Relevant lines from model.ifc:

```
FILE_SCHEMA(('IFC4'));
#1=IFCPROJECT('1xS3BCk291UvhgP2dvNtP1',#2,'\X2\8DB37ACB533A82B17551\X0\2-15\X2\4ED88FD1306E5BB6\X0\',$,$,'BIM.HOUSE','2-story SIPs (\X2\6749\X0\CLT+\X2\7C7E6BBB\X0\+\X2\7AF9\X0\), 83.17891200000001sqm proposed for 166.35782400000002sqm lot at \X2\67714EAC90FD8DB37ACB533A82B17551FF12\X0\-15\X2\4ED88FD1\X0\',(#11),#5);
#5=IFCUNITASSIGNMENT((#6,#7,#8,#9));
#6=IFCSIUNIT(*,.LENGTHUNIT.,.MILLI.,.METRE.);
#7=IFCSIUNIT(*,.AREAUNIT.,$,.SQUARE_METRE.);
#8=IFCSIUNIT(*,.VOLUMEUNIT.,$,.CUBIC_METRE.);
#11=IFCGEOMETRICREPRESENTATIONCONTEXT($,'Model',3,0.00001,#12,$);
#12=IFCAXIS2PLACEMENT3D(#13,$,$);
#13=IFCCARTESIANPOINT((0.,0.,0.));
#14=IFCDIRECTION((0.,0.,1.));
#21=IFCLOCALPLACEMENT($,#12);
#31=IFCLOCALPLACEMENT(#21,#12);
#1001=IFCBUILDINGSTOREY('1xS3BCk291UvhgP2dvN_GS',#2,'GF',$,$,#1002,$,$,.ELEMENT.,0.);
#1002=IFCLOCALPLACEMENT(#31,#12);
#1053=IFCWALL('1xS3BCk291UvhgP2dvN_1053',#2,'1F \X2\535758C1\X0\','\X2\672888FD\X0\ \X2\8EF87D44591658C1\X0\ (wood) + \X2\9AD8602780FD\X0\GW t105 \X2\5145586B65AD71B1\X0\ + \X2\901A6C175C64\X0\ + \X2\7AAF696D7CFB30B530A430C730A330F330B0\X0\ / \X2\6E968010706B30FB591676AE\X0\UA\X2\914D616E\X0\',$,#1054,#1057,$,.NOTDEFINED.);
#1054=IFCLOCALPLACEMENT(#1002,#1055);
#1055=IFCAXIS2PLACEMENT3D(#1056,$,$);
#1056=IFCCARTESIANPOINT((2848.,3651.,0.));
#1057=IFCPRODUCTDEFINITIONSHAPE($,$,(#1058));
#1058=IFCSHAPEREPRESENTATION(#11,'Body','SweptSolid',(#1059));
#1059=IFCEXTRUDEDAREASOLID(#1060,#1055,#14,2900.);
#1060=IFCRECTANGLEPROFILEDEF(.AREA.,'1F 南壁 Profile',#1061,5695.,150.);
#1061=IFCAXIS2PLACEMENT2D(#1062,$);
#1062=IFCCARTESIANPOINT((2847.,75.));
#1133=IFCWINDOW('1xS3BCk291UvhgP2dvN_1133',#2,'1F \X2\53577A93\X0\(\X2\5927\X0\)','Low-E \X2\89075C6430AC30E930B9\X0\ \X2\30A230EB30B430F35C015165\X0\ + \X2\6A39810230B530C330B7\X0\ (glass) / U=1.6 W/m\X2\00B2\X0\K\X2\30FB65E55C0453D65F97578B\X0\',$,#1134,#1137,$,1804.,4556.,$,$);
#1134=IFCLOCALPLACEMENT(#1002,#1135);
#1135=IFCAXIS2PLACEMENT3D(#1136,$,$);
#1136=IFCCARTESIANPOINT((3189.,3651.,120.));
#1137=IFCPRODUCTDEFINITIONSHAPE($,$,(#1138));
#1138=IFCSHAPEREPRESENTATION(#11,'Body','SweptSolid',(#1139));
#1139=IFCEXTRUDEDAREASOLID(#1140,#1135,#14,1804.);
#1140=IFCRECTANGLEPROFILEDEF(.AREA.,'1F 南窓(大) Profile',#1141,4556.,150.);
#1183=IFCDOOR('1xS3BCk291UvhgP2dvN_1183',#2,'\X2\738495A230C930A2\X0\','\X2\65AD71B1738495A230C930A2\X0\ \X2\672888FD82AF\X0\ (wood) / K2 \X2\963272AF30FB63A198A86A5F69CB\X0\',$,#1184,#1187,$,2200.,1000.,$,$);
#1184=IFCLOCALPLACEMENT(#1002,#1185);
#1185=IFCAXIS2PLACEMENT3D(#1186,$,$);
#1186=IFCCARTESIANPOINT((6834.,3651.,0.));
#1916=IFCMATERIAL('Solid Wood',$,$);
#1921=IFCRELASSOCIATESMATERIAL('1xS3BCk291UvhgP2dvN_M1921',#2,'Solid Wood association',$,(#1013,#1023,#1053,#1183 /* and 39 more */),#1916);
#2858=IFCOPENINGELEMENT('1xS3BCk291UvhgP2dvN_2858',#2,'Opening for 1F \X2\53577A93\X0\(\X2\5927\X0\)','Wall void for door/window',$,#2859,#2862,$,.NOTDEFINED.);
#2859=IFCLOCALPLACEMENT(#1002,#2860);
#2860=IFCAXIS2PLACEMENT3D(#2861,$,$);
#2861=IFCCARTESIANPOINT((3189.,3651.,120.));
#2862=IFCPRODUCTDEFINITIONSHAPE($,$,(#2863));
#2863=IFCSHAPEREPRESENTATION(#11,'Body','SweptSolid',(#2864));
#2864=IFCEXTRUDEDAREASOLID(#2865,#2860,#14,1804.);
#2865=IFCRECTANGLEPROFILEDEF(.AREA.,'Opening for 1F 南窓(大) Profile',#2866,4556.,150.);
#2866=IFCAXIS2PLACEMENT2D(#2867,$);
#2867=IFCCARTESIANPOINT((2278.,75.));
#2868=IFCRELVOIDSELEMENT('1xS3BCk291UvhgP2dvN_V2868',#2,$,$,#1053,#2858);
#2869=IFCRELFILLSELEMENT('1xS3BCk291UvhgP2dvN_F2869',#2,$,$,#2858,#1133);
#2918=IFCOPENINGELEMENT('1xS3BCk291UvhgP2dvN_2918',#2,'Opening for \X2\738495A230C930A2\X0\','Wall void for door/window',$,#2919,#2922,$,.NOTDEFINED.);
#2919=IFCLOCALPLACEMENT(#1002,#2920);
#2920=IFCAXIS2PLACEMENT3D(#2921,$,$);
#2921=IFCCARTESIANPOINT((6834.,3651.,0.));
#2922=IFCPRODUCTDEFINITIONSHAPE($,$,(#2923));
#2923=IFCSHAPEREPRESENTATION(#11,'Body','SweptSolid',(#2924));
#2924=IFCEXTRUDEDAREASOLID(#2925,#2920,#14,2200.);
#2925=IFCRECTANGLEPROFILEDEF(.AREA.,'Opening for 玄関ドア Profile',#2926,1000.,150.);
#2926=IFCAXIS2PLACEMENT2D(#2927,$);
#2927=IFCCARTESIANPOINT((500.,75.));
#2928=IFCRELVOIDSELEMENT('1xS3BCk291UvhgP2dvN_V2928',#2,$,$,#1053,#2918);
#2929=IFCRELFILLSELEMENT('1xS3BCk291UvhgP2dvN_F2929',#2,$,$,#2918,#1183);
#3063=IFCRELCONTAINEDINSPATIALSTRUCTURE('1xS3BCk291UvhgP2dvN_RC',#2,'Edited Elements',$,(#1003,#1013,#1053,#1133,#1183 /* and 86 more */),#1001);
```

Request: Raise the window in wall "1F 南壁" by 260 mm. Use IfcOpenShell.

```python
import numpy as np
import ifcopenshell
import ifcopenshell.api.geometry
import ifcopenshell.util.placement
import ifcopenshell.util.unit

model = ifcopenshell.open("model.ifc")
unit_scale = ifcopenshell.util.unit.calculate_unit_scale(model)

window = model.by_guid("1xS3BCk291UvhgP2dvN_1133")
opening = window.FillsVoids[0].RelatingOpeningElement
dz = 260.0

shift = np.array([0.0, 0.0, dz])
# The window is not placed relative to its opening, so move both.
for product in (opening, window):
    matrix = ifcopenshell.util.placement.get_local_placement(product.ObjectPlacement)
    matrix[:3, 3] += shift
    ifcopenshell.api.geometry.edit_object_placement(model, product=product, matrix=matrix, is_si=False)

print(f"moved by {dz * unit_scale:+.3f} m")

model.write("model-out.ifc")
```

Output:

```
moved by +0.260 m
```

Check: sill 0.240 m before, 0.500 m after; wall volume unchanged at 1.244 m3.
